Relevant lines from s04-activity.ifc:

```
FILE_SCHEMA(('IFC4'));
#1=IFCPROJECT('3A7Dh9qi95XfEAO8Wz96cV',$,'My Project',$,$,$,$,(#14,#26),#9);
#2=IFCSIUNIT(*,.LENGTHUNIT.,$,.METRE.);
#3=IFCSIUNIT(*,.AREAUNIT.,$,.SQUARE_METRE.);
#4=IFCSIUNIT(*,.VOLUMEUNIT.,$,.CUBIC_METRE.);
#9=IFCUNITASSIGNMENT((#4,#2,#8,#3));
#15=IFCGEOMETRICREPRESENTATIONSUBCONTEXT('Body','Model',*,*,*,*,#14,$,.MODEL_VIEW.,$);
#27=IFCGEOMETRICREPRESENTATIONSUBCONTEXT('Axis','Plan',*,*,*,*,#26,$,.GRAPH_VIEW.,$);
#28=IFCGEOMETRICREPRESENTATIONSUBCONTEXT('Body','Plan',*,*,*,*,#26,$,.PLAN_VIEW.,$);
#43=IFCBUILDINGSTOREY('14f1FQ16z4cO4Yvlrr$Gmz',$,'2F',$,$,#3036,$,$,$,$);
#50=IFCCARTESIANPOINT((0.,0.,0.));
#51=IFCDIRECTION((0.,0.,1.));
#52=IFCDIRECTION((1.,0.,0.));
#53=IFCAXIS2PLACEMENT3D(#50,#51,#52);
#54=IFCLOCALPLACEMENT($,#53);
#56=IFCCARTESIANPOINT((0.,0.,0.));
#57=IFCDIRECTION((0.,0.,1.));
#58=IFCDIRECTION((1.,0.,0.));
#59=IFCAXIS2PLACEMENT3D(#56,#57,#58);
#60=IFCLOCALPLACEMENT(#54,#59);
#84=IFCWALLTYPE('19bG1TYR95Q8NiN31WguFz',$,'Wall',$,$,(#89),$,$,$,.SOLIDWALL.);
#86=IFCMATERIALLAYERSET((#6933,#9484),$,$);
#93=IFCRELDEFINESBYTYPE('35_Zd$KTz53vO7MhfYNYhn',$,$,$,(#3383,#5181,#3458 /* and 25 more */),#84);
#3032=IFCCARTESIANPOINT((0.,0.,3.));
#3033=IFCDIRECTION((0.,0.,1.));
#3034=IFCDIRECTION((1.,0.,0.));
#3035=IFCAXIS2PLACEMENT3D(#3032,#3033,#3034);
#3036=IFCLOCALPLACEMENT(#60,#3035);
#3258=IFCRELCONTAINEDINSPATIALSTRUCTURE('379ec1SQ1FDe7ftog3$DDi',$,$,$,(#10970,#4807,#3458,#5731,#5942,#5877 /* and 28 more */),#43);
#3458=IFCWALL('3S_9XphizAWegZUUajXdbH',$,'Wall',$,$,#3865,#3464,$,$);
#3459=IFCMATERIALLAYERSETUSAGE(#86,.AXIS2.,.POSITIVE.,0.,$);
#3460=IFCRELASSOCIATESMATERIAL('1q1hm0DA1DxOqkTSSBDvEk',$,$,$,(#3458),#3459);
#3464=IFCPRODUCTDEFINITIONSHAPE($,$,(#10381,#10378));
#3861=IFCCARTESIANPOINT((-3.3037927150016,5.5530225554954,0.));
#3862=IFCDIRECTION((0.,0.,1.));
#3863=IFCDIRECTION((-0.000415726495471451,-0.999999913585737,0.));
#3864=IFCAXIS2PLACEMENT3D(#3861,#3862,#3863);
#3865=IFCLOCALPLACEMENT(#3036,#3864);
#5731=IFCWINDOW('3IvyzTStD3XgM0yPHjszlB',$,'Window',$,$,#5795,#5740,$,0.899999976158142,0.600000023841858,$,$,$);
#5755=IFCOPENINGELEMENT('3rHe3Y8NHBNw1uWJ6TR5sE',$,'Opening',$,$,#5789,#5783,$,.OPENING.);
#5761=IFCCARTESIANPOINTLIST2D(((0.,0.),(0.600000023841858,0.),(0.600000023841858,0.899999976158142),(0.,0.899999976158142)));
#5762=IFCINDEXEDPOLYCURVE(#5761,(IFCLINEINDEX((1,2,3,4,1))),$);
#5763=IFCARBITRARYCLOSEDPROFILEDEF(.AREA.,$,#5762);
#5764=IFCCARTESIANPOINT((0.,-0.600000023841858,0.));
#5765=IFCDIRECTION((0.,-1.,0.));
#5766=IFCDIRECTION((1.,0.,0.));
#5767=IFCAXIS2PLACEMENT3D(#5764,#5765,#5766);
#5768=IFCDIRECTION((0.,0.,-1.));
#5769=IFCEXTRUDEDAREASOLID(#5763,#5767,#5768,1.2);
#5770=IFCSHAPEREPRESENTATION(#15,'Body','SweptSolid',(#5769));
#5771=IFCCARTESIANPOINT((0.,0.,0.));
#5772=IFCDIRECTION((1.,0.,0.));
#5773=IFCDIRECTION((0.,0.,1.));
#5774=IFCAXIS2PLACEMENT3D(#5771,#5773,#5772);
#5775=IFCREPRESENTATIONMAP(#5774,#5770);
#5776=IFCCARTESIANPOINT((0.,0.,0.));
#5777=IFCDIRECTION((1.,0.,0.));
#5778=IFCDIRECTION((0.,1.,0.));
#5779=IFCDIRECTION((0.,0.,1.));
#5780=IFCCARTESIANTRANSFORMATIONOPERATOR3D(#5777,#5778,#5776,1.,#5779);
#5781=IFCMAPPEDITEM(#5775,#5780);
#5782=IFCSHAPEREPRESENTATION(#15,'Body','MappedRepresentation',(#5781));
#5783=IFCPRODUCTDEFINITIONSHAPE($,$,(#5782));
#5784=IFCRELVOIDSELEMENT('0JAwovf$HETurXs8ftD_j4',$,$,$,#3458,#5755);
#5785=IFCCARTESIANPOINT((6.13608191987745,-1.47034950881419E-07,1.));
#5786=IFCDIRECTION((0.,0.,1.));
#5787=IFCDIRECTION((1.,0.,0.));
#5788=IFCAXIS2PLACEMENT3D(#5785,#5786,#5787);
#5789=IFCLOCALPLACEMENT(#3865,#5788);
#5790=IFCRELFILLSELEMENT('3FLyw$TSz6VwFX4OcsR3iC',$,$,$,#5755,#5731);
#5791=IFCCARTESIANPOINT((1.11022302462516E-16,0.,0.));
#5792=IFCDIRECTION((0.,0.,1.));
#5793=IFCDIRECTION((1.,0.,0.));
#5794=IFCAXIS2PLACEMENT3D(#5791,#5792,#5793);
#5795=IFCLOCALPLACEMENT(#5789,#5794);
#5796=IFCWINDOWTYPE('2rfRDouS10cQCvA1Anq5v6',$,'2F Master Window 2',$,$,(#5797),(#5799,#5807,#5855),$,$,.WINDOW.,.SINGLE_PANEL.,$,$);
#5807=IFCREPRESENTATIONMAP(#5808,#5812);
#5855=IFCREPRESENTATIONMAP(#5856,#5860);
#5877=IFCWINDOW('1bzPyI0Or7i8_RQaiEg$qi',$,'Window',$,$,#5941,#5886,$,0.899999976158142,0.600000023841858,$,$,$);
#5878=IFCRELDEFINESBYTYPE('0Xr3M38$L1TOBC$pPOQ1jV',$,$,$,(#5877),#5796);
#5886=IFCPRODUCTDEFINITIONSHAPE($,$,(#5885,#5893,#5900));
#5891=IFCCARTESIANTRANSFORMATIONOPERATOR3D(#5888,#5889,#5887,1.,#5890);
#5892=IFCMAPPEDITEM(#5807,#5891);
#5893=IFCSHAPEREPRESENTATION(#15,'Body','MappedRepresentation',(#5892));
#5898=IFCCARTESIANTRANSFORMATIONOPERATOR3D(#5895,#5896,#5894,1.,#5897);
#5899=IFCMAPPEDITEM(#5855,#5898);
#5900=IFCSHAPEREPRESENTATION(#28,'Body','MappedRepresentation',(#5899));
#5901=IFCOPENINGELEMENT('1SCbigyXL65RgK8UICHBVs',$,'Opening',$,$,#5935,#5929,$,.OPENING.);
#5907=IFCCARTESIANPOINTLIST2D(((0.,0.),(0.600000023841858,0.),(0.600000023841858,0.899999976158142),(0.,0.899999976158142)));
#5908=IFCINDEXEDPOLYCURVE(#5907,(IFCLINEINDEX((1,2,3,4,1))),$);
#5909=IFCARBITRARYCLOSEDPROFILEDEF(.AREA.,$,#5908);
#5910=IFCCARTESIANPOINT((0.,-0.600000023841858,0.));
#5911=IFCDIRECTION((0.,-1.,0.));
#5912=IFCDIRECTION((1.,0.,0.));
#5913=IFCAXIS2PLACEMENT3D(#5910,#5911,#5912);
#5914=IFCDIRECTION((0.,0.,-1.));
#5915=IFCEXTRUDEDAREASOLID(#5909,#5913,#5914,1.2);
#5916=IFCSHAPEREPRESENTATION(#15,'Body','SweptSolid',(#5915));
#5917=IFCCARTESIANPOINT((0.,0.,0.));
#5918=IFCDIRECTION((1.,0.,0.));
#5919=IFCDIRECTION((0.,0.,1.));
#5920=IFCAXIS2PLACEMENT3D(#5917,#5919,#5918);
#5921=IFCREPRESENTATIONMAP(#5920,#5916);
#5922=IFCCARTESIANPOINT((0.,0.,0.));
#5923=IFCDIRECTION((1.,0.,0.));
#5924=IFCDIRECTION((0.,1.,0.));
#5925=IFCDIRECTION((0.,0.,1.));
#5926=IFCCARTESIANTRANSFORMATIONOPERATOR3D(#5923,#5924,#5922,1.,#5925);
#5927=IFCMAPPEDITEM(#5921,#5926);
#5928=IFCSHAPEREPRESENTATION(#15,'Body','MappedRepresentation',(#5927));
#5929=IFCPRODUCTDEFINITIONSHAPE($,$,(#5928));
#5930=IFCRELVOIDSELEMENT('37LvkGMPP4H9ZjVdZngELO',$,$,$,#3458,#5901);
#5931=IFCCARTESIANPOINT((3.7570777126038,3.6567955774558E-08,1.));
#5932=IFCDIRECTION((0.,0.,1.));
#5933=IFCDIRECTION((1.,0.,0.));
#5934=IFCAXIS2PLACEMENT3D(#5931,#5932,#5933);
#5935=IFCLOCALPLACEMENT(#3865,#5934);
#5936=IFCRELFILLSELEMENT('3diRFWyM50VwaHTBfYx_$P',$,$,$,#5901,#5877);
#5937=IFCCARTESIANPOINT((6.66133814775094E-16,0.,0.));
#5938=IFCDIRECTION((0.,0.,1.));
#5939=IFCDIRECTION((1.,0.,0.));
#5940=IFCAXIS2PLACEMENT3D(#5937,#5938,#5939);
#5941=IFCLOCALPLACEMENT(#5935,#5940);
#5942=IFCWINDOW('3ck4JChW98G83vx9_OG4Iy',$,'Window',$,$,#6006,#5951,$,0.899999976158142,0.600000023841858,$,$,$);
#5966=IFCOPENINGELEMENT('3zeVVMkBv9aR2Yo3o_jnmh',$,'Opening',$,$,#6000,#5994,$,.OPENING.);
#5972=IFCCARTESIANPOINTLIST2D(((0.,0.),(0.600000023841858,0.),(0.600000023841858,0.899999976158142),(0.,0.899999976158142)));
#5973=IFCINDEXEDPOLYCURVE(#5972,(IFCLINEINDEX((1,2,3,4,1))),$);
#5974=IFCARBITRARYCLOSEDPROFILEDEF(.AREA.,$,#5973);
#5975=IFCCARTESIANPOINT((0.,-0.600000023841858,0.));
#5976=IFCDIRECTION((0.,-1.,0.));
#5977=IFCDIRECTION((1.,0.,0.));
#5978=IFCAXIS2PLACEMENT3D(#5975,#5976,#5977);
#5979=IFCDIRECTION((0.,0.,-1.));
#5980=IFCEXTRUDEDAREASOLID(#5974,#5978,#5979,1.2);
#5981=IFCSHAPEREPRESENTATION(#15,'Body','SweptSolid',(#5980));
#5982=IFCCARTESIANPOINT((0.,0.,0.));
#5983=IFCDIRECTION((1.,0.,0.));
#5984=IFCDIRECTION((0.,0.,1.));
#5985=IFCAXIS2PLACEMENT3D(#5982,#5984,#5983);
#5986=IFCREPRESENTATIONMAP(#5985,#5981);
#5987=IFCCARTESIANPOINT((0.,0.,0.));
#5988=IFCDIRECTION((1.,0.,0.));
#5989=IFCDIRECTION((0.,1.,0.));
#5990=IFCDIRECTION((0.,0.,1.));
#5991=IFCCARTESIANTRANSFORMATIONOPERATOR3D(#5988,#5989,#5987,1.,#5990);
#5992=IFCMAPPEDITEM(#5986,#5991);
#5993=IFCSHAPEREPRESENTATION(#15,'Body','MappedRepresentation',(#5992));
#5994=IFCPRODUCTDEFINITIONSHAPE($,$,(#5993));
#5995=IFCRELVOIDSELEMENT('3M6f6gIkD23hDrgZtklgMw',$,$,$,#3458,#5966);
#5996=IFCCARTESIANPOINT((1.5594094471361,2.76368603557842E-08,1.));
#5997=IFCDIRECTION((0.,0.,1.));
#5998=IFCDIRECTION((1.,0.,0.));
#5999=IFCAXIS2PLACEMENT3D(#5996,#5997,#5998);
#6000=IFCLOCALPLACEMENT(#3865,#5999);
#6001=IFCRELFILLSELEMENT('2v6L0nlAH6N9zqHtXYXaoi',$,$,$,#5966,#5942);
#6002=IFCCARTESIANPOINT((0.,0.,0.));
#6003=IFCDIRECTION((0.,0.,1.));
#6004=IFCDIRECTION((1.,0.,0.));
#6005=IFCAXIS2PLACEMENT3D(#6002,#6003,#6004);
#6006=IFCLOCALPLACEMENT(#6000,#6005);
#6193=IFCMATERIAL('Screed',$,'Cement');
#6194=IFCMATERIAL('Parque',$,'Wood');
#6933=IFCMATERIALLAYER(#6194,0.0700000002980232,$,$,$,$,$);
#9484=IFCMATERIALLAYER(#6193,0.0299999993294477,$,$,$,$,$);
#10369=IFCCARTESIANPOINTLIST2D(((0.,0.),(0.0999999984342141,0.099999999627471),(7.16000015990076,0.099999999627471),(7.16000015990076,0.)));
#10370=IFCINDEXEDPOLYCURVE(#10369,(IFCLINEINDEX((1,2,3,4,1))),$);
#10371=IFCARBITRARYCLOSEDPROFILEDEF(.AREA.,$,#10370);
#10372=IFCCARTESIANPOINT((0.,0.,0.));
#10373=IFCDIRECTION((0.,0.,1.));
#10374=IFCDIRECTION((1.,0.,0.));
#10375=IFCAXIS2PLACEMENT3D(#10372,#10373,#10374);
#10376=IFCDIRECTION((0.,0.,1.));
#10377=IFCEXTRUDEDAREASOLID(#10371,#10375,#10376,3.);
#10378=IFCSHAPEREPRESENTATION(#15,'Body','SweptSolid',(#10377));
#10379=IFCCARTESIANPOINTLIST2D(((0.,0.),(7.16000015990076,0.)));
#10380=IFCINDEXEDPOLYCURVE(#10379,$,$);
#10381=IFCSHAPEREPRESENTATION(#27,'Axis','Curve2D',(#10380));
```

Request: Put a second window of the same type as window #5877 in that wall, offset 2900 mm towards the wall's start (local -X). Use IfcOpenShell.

```python
import ifcopenshell
import ifcopenshell.api.feature
import ifcopenshell.api.geometry
import ifcopenshell.api.root
import ifcopenshell.geom
import ifcopenshell.util.element
import ifcopenshell.util.placement
import ifcopenshell.util.shape

model = ifcopenshell.open("s04-activity.ifc")
settings = ifcopenshell.geom.settings()


def volume(element):
    """Net volume in cubic metres, openings subtracted."""
    shape = ifcopenshell.geom.create_shape(settings, element)
    return ifcopenshell.util.shape.get_volume(shape.geometry)


window = model.by_guid("1bzPyI0Or7i8_RQaiEg$qi")
opening = window.FillsVoids[0].RelatingOpeningElement
wall = opening.VoidsElements[0].RelatingBuildingElement
before = volume(wall)
shift = ifcopenshell.util.placement.get_local_placement(wall.ObjectPlacement)[:3, 0] * -2.9

# copy_class copies the void relationship, type, container and properties, but no geometry.
new_opening = ifcopenshell.api.root.copy_class(model, product=opening)
new_opening.Representation = ifcopenshell.util.element.copy_deep(
    model, opening.Representation, exclude=["IfcGeometricRepresentationContext", "IfcRepresentationMap"]
)
new_window = ifcopenshell.api.root.copy_class(model, product=window)
new_window.Representation = ifcopenshell.util.element.copy_deep(
    model, window.Representation, exclude=["IfcGeometricRepresentationContext", "IfcRepresentationMap"]
)
ifcopenshell.api.feature.add_filling(model, opening=new_opening, element=new_window)

for old, new in ((opening, new_opening), (window, new_window)):
    matrix = ifcopenshell.util.placement.get_local_placement(old.ObjectPlacement)
    matrix[:3, 3] += shift
    ifcopenshell.api.geometry.edit_object_placement(model, product=new, matrix=matrix, is_si=False)

after = volume(wall)

print(f"wall volume {before:.3f} -> {after:.3f} m3")

model.write("s04-activity-out.ifc")
```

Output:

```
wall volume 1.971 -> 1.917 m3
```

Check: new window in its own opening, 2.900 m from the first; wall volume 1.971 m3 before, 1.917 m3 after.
